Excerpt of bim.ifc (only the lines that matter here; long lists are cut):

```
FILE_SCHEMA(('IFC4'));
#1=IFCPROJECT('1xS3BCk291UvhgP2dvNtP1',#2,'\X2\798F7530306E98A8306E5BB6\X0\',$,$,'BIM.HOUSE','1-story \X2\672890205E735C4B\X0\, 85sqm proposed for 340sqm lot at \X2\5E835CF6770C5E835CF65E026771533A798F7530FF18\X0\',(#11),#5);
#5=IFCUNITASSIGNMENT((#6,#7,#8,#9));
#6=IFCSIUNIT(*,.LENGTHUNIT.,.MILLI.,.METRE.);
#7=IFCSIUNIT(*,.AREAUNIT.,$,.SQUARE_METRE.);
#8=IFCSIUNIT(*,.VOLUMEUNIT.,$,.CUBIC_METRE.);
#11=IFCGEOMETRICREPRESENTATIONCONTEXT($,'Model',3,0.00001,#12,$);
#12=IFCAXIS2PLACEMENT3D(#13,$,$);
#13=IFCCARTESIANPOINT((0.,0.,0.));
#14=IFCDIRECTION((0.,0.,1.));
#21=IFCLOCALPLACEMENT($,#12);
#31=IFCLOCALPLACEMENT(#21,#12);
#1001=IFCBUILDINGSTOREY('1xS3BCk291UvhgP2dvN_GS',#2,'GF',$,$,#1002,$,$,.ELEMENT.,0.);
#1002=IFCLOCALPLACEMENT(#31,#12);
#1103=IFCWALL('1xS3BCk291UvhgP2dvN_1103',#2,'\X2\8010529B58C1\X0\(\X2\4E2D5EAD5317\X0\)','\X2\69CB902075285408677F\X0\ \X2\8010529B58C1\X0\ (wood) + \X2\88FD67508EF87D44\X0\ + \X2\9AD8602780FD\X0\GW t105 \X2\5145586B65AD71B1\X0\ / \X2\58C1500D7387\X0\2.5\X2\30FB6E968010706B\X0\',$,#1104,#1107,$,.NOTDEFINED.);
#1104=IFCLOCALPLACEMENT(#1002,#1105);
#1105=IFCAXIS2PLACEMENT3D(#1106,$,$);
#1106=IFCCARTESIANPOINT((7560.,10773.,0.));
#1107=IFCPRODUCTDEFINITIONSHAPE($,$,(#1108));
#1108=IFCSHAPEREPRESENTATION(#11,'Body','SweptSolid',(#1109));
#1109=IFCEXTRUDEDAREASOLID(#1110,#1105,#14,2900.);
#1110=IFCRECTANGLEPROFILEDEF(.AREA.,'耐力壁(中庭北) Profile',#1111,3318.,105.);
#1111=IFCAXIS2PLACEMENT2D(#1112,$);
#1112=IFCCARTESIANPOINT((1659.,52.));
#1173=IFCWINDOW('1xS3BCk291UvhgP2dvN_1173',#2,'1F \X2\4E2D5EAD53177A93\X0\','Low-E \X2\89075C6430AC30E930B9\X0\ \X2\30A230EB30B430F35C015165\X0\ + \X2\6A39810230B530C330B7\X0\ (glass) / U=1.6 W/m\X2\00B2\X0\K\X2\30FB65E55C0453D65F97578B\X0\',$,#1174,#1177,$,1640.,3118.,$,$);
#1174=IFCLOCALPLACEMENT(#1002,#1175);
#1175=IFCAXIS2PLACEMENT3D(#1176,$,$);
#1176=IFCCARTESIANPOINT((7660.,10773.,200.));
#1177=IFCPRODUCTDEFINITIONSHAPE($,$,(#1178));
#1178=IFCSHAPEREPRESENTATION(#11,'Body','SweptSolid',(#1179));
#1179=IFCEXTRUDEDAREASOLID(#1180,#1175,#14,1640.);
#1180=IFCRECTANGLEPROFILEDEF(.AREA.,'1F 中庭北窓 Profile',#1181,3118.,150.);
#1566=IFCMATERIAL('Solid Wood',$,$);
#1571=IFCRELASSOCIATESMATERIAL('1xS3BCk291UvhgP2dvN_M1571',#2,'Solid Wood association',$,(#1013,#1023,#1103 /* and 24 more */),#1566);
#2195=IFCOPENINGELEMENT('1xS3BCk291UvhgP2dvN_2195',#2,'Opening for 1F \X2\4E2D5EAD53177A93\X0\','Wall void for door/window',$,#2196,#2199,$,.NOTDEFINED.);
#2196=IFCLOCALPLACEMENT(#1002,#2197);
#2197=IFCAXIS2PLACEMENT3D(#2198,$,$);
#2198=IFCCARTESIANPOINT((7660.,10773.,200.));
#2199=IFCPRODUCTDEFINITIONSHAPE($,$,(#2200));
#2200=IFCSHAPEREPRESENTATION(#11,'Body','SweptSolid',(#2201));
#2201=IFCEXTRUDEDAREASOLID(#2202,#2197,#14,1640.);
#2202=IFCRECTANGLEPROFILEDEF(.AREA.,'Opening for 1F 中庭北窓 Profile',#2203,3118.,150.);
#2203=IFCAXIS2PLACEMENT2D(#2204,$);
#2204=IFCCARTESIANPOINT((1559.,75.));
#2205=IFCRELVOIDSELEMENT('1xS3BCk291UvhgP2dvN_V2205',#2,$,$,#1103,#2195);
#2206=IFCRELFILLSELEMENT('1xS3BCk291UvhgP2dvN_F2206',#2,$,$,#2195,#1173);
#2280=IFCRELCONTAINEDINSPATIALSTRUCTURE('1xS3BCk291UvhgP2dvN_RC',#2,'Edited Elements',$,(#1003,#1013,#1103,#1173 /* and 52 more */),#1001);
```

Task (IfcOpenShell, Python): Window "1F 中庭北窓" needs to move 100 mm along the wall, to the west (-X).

```python
import ifcopenshell
import ifcopenshell.api.geometry
import ifcopenshell.util.placement
import ifcopenshell.util.unit

model = ifcopenshell.open("bim.ifc")
unit_scale = ifcopenshell.util.unit.calculate_unit_scale(model)

window = model.by_guid("1xS3BCk291UvhgP2dvN_1173")
opening = window.FillsVoids[0].RelatingOpeningElement
wall = opening.VoidsElements[0].RelatingBuildingElement

wall_matrix = ifcopenshell.util.placement.get_local_placement(wall.ObjectPlacement)
shift = wall_matrix[:3, 0] * -0.1 / unit_scale
before = ifcopenshell.util.placement.get_local_placement(window.ObjectPlacement)[:3, 3].copy()

# The window is not placed relative to its opening, so move both.
for product in (opening, window):
    matrix = ifcopenshell.util.placement.get_local_placement(product.ObjectPlacement)
    matrix[:3, 3] += shift
    ifcopenshell.api.geometry.edit_object_placement(model, product=product, matrix=matrix, is_si=False)

after = ifcopenshell.util.placement.get_local_placement(window.ObjectPlacement)[:3, 3]
print("window moved by", (after - before).round(3) + 0.0)

model.write("bim_rev.ifc")
```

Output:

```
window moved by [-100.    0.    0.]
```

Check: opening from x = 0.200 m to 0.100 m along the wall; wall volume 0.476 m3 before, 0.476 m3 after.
